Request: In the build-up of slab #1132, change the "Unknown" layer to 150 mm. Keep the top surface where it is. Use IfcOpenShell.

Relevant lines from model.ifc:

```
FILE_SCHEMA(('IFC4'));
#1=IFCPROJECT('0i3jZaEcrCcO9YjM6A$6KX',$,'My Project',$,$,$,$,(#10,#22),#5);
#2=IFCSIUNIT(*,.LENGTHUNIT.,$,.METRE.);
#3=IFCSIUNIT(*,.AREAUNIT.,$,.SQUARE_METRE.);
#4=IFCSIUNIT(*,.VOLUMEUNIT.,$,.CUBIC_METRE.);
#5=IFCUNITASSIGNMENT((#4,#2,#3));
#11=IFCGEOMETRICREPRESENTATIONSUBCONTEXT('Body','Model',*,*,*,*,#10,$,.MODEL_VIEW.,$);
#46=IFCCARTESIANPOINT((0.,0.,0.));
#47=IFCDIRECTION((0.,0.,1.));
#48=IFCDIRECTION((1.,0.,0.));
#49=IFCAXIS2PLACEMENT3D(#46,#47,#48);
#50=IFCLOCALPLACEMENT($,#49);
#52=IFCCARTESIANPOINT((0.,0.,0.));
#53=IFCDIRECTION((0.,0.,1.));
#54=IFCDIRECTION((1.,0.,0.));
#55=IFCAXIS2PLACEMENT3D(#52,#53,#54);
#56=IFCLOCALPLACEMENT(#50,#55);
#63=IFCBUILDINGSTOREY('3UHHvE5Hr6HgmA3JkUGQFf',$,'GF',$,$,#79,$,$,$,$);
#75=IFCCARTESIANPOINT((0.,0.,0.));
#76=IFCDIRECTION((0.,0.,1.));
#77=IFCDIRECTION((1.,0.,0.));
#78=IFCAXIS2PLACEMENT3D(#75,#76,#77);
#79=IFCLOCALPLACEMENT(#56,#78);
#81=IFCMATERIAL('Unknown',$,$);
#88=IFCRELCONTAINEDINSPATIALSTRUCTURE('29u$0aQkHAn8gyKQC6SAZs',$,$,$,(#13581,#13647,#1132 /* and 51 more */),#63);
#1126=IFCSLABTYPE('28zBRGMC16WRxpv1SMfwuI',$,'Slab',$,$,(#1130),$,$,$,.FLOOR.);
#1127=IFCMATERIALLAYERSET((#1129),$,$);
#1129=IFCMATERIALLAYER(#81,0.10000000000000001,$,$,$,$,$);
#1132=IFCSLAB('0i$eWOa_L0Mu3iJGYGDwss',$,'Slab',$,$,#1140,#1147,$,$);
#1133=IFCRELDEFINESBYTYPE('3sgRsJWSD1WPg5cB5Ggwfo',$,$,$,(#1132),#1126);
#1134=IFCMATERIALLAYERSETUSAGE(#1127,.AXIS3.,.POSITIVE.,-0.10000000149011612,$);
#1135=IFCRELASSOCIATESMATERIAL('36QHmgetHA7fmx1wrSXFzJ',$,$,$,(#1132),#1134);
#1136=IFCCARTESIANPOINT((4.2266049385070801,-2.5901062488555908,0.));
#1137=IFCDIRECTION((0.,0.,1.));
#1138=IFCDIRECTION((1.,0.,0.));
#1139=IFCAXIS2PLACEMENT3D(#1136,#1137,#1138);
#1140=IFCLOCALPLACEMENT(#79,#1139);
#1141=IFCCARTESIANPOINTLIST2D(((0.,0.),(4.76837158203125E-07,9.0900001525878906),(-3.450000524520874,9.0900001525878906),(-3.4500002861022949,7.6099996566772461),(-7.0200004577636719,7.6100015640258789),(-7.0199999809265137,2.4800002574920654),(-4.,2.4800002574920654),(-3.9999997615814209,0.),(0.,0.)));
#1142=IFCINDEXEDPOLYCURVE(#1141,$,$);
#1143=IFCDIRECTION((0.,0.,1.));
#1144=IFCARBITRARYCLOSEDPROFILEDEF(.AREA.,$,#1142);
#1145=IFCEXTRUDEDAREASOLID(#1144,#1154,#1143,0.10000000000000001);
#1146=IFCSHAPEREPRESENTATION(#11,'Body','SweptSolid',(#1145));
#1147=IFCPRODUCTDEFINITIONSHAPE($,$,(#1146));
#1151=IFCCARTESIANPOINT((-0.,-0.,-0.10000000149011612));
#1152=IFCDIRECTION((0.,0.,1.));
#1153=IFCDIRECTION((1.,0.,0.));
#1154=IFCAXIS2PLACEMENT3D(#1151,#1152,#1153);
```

```python
import ifcopenshell
import ifcopenshell.util.element
import ifcopenshell.util.representation

model = ifcopenshell.open("model.ifc")

layer_set = model.by_id(1127)
layer = next(l for l in layer_set.MaterialLayers if l.Material and l.Material.Name == "Unknown")
change = 0.15 - layer.LayerThickness
layer.LayerThickness += change

# Geometry does not follow the layer set by itself.
slabs = [e for e in ifcopenshell.util.element.get_elements_by_material(model, layer_set) if e.is_a("IfcSlab")]
for slab in sorted(slabs, key=lambda e: e.id()):
    body = ifcopenshell.util.representation.get_representation(slab, "Model", "Body")
    solid = body.Items[0]
    old_depth = solid.Depth
    solid.Depth += change
    # Extruded upwards: lower the start of the extrusion so the top stays.
    x, y, z = solid.Position.Location.Coordinates
    solid.Position.Location = model.createIfcCartesianPoint((x, y, z - change))
    print(slab.id(), f"{old_depth:g} -> {solid.Depth:g}")

# The layers are counted up from the underside, which has moved.
for usage in {ifcopenshell.util.element.get_material(slab) for slab in slabs}:
    usage.OffsetFromReferenceLine -= change

model.write("model_updated.ifc")
```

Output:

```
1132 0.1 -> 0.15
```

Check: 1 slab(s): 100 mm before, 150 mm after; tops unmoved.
